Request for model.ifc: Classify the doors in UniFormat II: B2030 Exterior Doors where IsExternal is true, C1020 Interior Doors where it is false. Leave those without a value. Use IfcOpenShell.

First a look at what the model holds.

```python
import ifcopenshell
import ifcopenshell.util.element

model = ifcopenshell.open("model.ifc")
print(model.schema)
print("classifications:", [c.Name for c in model.by_type("IfcClassification")])
values = [ifcopenshell.util.element.get_pset(e, "Pset_DoorCommon", "IsExternal") for e in model.by_type("IfcDoor")]
for value in (True, False, None):
    print("IsExternal", value, values.count(value))
```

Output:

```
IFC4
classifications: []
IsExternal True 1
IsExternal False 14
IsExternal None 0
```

```python
import ifcopenshell
import ifcopenshell.api.classification
import ifcopenshell.util.element

model = ifcopenshell.open("model.ifc")

system = ifcopenshell.api.classification.add_classification(model, classification="UniFormat II")

doors = model.by_type("IfcDoor")
external = {e: ifcopenshell.util.element.get_pset(e, "Pset_DoorCommon", "IsExternal") for e in doors}
for flag, code, name in ((True, "B2030", "Exterior Doors"), (False, "C1020", "Interior Doors")):
    products = [e for e in doors if external[e] is flag]
    ifcopenshell.api.classification.add_reference(
        model, products=products, classification=system, identification=code, name=name
    )
    print(code, len(products))

model.write("model_rev.ifc")
```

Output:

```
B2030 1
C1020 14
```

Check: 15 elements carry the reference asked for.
